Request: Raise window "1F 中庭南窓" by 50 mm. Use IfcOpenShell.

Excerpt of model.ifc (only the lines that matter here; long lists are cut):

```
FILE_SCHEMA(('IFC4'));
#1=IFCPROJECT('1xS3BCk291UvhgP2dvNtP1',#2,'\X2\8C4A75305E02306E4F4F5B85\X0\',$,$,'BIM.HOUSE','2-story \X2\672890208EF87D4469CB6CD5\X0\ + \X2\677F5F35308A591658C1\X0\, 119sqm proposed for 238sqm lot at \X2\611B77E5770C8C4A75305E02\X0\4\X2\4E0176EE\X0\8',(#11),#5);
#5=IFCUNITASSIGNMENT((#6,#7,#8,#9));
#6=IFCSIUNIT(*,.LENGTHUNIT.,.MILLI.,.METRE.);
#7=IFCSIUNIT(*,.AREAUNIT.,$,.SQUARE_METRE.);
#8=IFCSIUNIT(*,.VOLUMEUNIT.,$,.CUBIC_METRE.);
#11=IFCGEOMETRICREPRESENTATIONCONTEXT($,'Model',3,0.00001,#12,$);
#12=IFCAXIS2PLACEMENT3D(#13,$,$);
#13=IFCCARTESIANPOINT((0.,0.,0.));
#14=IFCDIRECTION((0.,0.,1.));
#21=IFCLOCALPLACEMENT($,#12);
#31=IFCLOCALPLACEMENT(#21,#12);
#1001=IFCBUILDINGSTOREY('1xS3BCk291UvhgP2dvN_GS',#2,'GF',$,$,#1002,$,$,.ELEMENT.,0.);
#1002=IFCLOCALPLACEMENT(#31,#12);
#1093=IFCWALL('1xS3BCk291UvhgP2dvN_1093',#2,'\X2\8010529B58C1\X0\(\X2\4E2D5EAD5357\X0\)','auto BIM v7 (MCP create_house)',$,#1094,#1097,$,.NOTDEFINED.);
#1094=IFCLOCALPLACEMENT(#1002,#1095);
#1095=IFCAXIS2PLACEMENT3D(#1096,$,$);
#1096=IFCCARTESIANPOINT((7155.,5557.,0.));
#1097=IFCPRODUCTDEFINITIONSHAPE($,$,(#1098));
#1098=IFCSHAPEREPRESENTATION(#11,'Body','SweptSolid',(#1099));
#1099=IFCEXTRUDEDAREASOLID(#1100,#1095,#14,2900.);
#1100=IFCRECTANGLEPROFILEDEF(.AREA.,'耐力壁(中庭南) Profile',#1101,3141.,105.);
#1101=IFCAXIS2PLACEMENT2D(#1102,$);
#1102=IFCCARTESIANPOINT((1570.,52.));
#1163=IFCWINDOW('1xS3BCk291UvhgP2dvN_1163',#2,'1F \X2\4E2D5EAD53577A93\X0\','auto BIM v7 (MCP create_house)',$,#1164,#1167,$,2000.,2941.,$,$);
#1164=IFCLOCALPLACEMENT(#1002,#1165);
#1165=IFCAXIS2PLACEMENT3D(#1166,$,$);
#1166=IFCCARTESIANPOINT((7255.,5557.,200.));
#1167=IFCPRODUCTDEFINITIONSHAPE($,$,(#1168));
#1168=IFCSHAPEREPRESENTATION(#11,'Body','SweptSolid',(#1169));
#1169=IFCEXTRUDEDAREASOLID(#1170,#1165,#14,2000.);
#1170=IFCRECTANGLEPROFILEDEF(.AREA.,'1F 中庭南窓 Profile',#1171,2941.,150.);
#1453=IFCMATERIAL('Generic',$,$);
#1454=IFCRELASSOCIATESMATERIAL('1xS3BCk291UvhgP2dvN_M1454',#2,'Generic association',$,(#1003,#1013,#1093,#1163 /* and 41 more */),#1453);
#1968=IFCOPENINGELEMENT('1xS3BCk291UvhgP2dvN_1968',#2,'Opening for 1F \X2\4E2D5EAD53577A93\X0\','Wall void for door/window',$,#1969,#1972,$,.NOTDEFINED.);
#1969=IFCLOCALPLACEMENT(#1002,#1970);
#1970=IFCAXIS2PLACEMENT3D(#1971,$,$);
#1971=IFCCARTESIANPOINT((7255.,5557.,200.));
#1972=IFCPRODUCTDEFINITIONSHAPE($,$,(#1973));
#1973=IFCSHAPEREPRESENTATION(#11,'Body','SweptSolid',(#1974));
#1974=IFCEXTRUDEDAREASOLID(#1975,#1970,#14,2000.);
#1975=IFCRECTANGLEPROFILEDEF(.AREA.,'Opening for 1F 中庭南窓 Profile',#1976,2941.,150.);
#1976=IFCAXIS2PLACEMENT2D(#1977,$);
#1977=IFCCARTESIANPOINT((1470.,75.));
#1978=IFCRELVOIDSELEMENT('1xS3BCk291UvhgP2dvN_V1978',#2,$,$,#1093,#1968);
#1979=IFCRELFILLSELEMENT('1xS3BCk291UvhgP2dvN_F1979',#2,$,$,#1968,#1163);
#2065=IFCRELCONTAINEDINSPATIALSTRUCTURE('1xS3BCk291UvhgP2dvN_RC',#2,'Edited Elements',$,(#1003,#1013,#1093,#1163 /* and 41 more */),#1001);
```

```python
import numpy as np
import ifcopenshell
import ifcopenshell.api.geometry
import ifcopenshell.util.placement
import ifcopenshell.util.unit

model = ifcopenshell.open("model.ifc")
unit_scale = ifcopenshell.util.unit.calculate_unit_scale(model)

window = model.by_id(1163)
opening = window.FillsVoids[0].RelatingOpeningElement
dz = 50.0

shift = np.array([0.0, 0.0, dz])
# The window is not placed relative to its opening, so move both.
for product in (opening, window):
    matrix = ifcopenshell.util.placement.get_local_placement(product.ObjectPlacement)
    matrix[:3, 3] += shift
    ifcopenshell.api.geometry.edit_object_placement(model, product=product, matrix=matrix, is_si=False)

print(f"moved by {dz * unit_scale:+.3f} m")

model.write("model_updated.ifc")
```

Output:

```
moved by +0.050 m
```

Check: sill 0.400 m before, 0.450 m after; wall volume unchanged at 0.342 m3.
